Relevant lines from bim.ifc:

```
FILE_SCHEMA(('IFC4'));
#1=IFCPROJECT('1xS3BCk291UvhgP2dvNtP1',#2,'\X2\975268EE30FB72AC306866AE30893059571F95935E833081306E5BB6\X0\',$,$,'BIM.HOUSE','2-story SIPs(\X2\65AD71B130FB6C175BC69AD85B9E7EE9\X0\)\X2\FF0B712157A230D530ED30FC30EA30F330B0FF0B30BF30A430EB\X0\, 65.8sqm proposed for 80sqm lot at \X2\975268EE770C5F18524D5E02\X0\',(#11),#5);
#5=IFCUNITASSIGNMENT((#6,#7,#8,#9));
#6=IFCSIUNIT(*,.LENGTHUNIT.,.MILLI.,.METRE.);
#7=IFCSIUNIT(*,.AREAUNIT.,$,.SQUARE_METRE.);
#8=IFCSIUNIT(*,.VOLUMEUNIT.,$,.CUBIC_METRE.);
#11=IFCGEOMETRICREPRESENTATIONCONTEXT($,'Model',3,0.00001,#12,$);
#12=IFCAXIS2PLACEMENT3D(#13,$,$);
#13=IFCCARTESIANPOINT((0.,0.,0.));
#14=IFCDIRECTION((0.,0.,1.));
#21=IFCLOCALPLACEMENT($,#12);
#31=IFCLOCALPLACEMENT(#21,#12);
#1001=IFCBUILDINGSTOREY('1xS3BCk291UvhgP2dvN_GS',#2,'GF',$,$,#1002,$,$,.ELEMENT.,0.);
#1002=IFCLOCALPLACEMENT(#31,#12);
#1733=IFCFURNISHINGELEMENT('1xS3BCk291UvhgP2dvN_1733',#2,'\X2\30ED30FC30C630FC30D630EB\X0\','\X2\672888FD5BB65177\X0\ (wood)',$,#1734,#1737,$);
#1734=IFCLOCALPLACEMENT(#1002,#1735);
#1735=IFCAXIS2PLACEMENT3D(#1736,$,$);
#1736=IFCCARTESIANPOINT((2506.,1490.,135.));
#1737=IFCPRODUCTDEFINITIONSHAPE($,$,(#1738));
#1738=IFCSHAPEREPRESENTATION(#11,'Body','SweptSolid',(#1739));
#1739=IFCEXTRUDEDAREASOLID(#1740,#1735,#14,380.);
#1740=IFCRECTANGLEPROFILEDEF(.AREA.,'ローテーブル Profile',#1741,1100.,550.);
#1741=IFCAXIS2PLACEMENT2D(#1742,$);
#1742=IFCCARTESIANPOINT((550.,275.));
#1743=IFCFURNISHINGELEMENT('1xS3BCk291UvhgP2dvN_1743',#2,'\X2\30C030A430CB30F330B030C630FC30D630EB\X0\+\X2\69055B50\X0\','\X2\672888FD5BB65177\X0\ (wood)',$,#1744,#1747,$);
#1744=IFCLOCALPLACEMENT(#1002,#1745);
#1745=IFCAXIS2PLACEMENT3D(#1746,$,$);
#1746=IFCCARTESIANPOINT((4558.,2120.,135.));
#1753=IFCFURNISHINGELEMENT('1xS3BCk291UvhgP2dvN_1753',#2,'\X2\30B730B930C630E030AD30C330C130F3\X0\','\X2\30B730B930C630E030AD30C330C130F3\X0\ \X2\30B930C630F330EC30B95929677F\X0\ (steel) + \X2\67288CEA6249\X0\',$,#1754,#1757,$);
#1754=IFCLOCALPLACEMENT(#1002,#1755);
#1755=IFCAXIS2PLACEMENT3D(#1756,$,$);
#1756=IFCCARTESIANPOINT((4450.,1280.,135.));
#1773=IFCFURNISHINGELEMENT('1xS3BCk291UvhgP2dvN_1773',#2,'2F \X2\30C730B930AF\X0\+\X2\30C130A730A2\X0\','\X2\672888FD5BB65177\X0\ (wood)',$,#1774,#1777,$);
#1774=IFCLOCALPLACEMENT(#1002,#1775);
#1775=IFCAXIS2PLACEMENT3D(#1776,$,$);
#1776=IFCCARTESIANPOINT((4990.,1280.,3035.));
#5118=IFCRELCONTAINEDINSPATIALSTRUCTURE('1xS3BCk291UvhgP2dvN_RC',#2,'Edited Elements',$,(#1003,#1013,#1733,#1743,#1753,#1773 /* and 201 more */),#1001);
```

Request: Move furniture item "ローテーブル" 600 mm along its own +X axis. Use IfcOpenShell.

```python
import ifcopenshell
import ifcopenshell.api.geometry
import ifcopenshell.util.placement

model = ifcopenshell.open("bim.ifc")

item = model.by_guid("1xS3BCk291UvhgP2dvN_1733")
matrix = ifcopenshell.util.placement.get_local_placement(item.ObjectPlacement)
matrix[:3, 3] += matrix[:3, 0] * 600.0
ifcopenshell.api.geometry.edit_object_placement(model, product=item, matrix=matrix, is_si=False)

print(ifcopenshell.util.placement.get_local_placement(item.ObjectPlacement).round(3) + 0.0)

model.write("bim-out.ifc")
```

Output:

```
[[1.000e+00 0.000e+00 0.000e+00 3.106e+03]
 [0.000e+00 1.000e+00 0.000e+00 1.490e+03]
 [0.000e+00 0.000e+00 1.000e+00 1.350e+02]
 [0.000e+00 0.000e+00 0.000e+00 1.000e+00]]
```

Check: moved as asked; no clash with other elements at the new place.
